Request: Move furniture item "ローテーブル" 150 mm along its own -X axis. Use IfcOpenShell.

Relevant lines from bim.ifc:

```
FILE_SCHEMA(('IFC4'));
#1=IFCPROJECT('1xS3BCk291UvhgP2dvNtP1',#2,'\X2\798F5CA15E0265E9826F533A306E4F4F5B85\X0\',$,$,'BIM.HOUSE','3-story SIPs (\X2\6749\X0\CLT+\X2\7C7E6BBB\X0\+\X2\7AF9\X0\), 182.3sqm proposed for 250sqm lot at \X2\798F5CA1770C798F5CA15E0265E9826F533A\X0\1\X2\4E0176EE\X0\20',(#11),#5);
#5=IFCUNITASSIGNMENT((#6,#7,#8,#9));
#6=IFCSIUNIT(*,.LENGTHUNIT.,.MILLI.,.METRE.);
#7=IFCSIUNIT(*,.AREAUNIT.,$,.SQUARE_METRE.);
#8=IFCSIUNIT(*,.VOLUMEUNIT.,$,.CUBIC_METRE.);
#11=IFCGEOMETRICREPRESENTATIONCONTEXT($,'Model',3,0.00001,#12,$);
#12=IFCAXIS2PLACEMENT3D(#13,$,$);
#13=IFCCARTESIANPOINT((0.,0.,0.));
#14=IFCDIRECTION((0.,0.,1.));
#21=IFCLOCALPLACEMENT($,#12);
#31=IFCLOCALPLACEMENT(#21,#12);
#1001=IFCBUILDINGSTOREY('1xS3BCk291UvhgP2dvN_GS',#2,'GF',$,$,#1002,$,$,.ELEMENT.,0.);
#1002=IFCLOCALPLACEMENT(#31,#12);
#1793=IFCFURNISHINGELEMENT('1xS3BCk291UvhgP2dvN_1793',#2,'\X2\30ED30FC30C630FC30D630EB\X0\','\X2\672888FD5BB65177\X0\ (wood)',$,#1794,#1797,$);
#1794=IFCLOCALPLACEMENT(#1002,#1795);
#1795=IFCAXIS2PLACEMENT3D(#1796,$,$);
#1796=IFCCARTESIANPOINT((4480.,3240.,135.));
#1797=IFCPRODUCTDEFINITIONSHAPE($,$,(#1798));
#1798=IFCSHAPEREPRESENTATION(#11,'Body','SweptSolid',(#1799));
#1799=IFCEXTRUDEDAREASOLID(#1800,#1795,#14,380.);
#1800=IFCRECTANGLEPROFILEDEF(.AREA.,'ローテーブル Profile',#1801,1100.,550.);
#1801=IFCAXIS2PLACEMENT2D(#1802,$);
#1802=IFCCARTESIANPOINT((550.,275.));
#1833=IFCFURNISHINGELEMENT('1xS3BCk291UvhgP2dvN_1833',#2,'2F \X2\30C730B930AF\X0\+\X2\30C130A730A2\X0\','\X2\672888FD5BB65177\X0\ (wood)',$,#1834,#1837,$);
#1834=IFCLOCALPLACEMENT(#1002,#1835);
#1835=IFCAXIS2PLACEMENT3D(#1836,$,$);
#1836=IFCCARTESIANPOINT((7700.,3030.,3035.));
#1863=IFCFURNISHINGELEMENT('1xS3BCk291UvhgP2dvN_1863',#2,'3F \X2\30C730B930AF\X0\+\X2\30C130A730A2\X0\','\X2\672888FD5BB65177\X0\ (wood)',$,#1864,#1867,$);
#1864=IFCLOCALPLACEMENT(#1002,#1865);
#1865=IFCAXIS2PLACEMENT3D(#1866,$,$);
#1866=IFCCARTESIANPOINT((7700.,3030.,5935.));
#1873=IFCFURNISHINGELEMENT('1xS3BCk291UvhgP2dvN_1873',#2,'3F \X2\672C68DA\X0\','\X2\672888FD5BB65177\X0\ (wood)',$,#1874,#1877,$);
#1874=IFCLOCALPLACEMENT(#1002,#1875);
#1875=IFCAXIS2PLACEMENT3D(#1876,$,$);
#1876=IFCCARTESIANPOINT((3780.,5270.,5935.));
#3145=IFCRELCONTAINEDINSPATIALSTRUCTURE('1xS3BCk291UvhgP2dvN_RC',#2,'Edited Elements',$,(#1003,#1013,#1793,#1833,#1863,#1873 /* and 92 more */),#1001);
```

```python
import ifcopenshell
import ifcopenshell.api.geometry
import ifcopenshell.util.placement
import ifcopenshell.util.unit

model = ifcopenshell.open("bim.ifc")
unit_scale = ifcopenshell.util.unit.calculate_unit_scale(model)

item = model.by_id(1793)
matrix = ifcopenshell.util.placement.get_local_placement(item.ObjectPlacement)
matrix[:3, 3] -= matrix[:3, 0] * 0.15 / unit_scale
ifcopenshell.api.geometry.edit_object_placement(model, product=item, matrix=matrix, is_si=False)

print(ifcopenshell.util.placement.get_local_placement(item.ObjectPlacement).round(3) + 0.0)

model.write("bim_v2.ifc")
```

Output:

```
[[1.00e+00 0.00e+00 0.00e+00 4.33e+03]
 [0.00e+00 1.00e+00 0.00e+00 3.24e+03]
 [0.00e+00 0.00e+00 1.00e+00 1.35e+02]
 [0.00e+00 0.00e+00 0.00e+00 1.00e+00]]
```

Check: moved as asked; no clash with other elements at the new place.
